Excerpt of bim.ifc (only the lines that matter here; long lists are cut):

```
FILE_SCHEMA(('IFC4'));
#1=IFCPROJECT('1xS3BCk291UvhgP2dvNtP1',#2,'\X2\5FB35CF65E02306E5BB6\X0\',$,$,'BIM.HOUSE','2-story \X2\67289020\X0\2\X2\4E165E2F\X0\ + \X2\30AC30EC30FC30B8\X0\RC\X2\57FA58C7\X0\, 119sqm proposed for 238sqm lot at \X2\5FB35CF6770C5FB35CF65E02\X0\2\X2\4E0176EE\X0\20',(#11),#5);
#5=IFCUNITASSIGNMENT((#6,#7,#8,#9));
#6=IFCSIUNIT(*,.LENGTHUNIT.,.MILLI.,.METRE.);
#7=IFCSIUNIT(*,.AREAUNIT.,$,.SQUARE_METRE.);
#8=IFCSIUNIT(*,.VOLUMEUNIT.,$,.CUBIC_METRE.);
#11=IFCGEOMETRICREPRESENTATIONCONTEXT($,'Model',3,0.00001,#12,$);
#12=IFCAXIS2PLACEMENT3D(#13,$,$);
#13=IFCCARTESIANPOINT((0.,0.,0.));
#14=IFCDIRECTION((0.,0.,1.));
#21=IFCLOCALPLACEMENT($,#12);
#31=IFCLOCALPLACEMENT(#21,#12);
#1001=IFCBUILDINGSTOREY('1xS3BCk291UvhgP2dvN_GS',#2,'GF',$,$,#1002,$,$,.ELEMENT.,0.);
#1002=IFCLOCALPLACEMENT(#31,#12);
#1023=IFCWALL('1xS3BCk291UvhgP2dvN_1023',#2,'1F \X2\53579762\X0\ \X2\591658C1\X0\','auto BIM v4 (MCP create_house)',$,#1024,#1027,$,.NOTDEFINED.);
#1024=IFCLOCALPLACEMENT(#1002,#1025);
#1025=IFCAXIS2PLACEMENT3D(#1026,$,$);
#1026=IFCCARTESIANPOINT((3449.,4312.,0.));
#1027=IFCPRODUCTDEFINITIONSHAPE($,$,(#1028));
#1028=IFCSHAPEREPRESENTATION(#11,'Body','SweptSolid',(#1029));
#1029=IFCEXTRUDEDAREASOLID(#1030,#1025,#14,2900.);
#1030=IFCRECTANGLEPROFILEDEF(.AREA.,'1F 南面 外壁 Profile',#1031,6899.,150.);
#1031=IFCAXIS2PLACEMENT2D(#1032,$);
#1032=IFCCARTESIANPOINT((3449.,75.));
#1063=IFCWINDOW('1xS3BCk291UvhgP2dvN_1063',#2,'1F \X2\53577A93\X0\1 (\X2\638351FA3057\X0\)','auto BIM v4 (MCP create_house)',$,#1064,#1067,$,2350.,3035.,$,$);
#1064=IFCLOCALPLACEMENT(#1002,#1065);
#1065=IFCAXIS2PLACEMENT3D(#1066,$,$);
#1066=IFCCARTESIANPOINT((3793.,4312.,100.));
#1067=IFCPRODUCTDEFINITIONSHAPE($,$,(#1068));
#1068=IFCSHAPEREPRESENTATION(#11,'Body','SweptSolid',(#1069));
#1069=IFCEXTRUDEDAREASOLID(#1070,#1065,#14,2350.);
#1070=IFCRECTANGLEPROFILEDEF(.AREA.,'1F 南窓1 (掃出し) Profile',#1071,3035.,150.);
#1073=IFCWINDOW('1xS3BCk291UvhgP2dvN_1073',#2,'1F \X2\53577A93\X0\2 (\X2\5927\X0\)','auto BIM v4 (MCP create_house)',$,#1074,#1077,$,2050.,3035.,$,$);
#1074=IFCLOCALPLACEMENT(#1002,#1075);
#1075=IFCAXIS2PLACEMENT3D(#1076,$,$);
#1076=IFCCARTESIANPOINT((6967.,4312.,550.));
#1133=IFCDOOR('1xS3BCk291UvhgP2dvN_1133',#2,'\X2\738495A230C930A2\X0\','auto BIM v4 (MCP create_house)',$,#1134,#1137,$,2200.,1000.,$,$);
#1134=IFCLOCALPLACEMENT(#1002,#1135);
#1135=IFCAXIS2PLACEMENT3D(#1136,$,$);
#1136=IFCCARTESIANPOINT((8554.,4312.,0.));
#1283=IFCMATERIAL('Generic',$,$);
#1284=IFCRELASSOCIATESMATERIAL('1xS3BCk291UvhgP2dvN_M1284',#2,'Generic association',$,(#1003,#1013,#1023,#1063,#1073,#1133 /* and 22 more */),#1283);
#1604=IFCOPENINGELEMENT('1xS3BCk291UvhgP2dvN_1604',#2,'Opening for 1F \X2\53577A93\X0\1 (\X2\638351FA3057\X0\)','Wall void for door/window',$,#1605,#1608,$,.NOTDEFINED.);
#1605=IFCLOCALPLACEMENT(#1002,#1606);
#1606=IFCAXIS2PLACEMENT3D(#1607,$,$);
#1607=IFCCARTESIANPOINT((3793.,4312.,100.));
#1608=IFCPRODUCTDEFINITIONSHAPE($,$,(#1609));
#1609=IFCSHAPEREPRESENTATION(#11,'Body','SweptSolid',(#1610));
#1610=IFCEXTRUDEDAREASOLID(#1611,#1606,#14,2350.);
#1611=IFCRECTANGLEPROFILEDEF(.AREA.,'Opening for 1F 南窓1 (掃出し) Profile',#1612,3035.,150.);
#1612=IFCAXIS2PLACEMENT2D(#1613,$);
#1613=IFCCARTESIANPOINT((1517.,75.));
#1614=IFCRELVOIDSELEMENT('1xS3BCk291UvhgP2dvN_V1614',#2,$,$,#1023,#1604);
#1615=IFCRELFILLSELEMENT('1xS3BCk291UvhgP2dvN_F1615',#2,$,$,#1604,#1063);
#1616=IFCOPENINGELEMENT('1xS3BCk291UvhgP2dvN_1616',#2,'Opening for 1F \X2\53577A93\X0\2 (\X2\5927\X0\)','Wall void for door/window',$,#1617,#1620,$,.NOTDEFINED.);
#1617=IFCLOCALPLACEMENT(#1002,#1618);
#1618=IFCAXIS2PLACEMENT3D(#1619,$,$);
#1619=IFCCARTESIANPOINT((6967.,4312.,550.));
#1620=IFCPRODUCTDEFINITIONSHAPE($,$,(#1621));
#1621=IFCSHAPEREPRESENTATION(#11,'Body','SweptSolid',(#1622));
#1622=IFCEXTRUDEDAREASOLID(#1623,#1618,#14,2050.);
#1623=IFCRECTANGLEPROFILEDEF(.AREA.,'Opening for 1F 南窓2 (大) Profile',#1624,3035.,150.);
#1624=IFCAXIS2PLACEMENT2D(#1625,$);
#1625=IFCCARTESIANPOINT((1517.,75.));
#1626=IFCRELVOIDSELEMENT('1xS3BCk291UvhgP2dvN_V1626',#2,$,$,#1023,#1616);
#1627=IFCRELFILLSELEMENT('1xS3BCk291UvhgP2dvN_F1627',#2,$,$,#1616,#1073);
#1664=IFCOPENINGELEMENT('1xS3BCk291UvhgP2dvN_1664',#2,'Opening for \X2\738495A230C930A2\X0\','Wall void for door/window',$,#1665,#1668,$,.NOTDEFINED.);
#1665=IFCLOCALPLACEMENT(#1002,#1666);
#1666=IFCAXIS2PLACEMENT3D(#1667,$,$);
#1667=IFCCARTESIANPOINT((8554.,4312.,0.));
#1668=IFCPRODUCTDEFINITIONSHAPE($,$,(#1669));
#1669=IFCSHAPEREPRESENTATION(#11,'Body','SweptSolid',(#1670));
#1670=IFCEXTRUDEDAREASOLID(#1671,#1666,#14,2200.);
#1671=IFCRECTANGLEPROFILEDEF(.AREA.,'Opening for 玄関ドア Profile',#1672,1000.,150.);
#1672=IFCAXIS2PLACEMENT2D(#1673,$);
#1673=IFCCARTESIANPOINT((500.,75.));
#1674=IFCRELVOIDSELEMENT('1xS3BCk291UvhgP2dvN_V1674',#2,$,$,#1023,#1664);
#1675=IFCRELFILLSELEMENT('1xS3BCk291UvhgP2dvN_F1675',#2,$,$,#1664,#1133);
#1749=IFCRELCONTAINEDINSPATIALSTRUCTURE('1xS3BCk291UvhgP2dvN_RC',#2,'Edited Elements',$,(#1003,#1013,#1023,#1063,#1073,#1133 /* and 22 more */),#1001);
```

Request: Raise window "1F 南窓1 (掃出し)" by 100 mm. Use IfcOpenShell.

```python
import numpy as np
import ifcopenshell
import ifcopenshell.api.geometry
import ifcopenshell.util.placement
import ifcopenshell.util.unit

model = ifcopenshell.open("bim.ifc")
unit_scale = ifcopenshell.util.unit.calculate_unit_scale(model)

window = model.by_id(1063)
opening = window.FillsVoids[0].RelatingOpeningElement
dz = 0.1 / unit_scale

shift = np.array([0.0, 0.0, dz])
# The window is not placed relative to its opening, so move both.
for product in (opening, window):
    matrix = ifcopenshell.util.placement.get_local_placement(product.ObjectPlacement)
    matrix[:3, 3] += shift
    ifcopenshell.api.geometry.edit_object_placement(model, product=product, matrix=matrix, is_si=False)

print(f"moved by {dz * unit_scale:+.3f} m")

model.write("bim-out.ifc")
```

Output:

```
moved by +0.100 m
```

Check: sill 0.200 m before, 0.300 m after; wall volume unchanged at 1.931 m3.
